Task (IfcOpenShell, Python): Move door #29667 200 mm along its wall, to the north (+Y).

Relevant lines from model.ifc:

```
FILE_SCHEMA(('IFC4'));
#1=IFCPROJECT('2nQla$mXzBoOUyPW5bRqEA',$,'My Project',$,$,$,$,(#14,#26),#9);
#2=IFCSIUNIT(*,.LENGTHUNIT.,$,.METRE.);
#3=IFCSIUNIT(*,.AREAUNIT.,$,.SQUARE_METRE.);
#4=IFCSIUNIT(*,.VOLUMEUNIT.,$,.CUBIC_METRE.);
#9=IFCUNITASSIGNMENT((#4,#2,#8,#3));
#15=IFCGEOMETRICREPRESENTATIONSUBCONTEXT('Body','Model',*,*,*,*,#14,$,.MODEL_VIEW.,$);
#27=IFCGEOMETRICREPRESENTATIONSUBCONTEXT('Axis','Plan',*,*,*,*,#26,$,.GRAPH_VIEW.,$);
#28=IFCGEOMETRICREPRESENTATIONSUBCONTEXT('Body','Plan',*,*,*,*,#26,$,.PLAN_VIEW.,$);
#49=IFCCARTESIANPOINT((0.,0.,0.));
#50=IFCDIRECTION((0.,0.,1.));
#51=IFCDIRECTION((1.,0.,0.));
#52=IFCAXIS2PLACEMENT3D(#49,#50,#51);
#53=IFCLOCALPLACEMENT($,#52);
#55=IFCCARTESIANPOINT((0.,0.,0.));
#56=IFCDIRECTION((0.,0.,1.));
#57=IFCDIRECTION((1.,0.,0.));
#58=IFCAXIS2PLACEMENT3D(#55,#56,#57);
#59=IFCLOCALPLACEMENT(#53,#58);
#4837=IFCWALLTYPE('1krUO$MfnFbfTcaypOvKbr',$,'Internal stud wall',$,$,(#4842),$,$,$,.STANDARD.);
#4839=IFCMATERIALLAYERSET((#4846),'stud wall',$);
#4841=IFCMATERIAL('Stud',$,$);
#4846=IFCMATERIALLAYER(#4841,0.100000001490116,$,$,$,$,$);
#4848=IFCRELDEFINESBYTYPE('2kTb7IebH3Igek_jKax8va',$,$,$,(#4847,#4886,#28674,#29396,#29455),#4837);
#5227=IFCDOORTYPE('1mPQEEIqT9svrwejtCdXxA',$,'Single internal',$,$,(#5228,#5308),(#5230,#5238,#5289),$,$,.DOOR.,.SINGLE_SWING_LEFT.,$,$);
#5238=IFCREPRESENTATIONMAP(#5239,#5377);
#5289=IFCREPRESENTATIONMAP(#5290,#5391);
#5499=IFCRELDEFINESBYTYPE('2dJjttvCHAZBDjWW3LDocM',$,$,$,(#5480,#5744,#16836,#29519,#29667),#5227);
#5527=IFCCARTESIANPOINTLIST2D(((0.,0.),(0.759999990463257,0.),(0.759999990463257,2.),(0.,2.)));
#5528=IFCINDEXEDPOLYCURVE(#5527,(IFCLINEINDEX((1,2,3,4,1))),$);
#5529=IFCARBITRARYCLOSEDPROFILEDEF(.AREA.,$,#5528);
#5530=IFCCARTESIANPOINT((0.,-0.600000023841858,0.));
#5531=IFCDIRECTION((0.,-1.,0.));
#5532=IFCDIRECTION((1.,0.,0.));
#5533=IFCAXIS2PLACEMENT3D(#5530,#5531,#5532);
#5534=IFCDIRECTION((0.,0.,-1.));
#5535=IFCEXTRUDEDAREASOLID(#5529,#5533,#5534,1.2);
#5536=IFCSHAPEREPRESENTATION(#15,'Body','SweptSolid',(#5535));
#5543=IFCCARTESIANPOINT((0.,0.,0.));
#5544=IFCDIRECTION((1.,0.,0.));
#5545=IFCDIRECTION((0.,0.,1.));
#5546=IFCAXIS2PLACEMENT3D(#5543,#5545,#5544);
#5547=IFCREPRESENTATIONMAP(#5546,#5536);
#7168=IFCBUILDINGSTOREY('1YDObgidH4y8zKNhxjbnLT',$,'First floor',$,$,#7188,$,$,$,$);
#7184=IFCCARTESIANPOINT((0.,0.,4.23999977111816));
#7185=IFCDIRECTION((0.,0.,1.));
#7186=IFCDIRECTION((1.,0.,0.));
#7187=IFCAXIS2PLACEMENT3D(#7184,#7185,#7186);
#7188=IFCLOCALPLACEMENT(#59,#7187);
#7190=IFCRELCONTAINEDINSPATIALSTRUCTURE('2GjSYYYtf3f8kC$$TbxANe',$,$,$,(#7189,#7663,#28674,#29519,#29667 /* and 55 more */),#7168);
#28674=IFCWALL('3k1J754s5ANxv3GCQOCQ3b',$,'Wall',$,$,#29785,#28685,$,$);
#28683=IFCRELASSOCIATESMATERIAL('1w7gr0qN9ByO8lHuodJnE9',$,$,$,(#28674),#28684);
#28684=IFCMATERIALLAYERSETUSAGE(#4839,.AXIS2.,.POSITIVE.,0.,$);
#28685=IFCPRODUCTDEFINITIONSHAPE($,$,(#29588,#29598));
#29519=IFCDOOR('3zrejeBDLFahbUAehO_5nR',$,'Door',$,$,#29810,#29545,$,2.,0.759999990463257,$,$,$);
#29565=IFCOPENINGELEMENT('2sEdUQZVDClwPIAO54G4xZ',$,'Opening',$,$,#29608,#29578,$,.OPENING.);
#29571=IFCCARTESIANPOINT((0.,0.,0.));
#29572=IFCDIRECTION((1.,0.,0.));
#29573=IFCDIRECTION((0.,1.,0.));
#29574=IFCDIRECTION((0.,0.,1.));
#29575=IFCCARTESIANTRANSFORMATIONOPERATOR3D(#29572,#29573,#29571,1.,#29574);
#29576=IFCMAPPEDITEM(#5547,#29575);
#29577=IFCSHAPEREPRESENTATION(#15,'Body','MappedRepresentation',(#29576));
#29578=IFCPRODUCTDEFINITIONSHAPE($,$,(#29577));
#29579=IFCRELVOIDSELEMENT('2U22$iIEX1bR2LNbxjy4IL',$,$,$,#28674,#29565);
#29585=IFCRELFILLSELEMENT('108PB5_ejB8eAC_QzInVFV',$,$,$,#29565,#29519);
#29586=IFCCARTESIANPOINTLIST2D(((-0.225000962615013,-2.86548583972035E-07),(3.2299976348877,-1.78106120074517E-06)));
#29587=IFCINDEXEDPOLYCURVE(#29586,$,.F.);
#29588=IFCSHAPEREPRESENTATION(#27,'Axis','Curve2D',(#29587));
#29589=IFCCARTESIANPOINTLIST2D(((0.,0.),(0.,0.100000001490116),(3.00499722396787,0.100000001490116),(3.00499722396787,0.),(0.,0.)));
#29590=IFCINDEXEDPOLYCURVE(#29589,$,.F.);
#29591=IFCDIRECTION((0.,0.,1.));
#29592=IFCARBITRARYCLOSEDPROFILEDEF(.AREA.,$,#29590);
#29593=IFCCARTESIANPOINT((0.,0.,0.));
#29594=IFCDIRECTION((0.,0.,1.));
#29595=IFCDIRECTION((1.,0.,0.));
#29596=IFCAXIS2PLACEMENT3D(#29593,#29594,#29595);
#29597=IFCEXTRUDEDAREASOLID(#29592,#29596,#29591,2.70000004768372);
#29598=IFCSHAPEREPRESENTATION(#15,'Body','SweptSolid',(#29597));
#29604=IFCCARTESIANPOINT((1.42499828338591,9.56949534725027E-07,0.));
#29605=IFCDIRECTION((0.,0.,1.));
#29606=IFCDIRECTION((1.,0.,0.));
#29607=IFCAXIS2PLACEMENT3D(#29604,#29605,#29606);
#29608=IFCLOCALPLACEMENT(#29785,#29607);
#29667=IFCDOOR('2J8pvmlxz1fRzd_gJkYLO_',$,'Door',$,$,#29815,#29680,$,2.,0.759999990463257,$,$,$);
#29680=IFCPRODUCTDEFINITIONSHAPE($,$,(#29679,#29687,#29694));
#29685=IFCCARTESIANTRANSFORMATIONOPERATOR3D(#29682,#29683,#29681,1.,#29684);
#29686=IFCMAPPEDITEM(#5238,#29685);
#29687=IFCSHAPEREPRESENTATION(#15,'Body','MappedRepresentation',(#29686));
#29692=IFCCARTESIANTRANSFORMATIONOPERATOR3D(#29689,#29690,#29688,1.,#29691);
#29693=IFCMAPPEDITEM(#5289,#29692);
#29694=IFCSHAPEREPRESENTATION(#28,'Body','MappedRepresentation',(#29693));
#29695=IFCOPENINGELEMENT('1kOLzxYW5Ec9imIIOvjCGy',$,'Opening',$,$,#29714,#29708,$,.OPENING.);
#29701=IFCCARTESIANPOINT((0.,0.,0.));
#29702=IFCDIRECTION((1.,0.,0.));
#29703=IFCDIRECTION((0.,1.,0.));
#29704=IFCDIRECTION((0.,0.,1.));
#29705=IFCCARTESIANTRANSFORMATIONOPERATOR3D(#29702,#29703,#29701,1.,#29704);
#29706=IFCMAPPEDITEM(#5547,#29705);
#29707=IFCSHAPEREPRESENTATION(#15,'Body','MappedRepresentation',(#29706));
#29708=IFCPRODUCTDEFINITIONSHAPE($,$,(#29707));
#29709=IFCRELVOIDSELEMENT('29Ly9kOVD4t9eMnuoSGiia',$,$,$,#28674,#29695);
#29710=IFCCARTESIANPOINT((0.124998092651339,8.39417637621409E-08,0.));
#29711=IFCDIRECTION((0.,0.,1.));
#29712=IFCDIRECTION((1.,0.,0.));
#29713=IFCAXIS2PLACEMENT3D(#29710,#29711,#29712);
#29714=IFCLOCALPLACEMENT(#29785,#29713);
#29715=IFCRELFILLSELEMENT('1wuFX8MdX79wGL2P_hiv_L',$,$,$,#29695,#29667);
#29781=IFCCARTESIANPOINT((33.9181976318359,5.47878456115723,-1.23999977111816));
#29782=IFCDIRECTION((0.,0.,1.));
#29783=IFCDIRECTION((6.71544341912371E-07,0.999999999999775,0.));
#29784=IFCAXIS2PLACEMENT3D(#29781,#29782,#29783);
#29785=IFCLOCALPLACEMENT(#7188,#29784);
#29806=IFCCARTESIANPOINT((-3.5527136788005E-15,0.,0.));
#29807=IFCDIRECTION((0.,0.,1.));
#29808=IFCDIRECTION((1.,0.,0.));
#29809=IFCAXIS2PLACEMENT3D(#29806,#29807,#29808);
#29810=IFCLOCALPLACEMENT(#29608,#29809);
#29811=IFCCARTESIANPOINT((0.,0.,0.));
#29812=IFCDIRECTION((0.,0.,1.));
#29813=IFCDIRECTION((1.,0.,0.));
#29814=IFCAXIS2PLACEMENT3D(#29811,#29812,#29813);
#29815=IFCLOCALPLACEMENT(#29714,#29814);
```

```python
import ifcopenshell
import ifcopenshell.api.geometry
import ifcopenshell.util.placement
import ifcopenshell.util.unit

model = ifcopenshell.open("model.ifc")
unit_scale = ifcopenshell.util.unit.calculate_unit_scale(model)

door = model.by_id(29667)
opening = door.FillsVoids[0].RelatingOpeningElement
wall = opening.VoidsElements[0].RelatingBuildingElement

wall_matrix = ifcopenshell.util.placement.get_local_placement(wall.ObjectPlacement)
shift = wall_matrix[:3, 0] * 0.2 / unit_scale
before = ifcopenshell.util.placement.get_local_placement(door.ObjectPlacement)[:3, 3].copy()

# The door is placed relative to its opening, so it follows when the opening moves.
matrix = ifcopenshell.util.placement.get_local_placement(opening.ObjectPlacement)
matrix[:3, 3] += shift
ifcopenshell.api.geometry.edit_object_placement(
    model, product=opening, matrix=matrix, is_si=False, should_transform_children=True
)

after = ifcopenshell.util.placement.get_local_placement(door.ObjectPlacement)[:3, 3]
print("door moved by", (after - before).round(3) + 0.0)

model.write("model_v2.ifc")
```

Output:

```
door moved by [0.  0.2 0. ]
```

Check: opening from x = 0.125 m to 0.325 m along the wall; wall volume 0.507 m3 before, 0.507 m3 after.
